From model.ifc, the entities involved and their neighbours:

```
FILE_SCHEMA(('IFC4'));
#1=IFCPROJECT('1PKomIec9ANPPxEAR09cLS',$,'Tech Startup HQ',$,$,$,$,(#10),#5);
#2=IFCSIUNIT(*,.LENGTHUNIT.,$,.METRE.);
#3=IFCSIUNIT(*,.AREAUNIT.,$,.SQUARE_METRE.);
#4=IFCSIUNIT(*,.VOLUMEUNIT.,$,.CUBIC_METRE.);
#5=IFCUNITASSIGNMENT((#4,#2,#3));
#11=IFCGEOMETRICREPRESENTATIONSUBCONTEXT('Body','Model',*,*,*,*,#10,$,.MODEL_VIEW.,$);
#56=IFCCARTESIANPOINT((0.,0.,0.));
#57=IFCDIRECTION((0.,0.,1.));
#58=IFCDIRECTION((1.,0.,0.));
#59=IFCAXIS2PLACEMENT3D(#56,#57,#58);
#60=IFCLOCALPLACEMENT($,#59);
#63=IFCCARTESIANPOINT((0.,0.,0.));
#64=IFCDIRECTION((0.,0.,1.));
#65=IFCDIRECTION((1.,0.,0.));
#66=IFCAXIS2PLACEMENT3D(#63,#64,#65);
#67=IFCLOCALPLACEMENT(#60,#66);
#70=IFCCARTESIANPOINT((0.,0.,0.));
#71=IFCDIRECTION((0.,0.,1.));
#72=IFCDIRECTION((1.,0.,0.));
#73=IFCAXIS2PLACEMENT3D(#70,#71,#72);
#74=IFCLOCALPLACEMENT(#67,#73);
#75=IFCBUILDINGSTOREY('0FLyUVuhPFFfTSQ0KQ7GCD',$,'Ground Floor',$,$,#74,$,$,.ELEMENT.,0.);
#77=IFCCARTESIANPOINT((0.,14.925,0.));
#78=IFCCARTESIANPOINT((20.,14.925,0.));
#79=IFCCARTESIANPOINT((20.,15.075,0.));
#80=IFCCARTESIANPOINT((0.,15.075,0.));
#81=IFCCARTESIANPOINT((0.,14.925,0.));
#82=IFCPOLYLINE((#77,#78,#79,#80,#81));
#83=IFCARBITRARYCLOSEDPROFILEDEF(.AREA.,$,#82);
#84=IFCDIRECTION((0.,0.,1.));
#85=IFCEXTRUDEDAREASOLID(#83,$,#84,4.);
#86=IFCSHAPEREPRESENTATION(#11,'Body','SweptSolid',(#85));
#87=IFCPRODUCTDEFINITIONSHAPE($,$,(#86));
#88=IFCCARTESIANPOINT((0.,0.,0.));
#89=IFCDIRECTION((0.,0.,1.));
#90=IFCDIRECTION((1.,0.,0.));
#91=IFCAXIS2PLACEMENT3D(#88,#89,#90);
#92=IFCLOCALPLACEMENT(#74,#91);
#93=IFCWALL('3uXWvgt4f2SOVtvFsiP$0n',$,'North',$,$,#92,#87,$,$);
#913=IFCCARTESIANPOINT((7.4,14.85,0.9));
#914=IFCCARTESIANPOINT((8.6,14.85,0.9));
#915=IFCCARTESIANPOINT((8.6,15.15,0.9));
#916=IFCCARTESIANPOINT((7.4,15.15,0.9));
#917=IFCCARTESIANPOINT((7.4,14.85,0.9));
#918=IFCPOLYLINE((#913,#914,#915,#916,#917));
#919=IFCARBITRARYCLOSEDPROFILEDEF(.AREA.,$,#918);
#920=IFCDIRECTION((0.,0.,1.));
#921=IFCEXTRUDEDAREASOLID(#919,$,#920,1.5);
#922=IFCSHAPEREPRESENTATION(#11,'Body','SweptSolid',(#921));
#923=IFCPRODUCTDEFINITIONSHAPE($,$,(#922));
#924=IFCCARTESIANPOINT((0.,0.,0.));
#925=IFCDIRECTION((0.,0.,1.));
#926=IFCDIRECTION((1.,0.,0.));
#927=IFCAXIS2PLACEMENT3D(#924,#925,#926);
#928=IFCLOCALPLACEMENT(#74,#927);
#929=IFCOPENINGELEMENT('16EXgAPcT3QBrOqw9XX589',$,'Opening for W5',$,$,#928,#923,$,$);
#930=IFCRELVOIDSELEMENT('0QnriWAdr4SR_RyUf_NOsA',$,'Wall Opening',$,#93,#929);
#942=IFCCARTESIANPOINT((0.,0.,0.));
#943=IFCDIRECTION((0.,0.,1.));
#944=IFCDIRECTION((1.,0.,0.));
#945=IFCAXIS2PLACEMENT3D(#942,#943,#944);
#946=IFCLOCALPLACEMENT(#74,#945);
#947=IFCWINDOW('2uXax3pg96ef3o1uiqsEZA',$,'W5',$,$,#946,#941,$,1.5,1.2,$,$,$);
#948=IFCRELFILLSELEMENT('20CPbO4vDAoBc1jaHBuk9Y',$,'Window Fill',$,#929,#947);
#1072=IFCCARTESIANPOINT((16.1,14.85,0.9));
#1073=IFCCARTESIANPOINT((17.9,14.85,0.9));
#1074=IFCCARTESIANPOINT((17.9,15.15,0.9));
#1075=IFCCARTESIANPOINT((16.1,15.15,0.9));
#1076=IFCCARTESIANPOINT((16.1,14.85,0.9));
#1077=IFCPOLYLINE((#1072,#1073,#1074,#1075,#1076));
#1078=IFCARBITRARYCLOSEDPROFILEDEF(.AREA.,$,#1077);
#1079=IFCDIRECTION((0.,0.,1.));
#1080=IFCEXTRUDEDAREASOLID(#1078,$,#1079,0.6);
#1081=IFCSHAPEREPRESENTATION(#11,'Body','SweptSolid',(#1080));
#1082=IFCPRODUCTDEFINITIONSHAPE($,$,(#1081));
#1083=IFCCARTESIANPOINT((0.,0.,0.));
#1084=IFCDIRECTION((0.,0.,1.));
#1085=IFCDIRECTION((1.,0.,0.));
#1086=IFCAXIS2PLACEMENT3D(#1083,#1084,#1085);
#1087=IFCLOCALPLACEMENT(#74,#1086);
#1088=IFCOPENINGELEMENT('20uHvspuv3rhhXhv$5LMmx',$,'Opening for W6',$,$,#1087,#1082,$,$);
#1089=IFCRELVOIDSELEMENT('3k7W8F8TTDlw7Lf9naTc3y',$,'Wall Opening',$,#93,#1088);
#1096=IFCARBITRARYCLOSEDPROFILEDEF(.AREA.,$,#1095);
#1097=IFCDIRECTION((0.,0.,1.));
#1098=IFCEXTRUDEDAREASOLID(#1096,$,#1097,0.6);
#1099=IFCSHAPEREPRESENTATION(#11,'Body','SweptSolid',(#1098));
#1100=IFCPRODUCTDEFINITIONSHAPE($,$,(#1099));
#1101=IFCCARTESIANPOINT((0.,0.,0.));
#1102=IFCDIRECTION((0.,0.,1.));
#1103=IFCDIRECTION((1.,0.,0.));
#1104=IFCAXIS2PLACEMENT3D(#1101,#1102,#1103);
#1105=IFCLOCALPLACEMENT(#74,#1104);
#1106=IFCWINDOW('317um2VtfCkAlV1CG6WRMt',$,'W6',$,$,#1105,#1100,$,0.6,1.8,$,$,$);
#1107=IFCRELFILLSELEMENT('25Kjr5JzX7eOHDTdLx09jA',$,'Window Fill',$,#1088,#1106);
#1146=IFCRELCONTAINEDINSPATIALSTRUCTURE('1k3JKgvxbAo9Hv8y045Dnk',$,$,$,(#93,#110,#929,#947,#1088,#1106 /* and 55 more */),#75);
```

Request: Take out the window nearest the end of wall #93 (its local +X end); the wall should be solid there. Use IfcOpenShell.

```python
import ifcopenshell
import ifcopenshell.api.feature
import ifcopenshell.api.root
import ifcopenshell.geom
import ifcopenshell.util.shape

model = ifcopenshell.open("model.ifc")
settings = ifcopenshell.geom.settings()


def volume(element):
    """Net volume in cubic metres, openings subtracted."""
    shape = ifcopenshell.geom.create_shape(settings, element)
    return ifcopenshell.util.shape.get_volume(shape.geometry)


window = model.by_guid("317um2VtfCkAlV1CG6WRMt")
opening = window.FillsVoids[0].RelatingOpeningElement
wall = opening.VoidsElements[0].RelatingBuildingElement
before = volume(wall)

ifcopenshell.api.root.remove_product(model, product=window)
ifcopenshell.api.feature.remove_feature(model, feature=opening)

after = volume(wall)

print(f"wall volume {before:.3f} -> {after:.3f} m3")

model.write("model_v2.ifc")
```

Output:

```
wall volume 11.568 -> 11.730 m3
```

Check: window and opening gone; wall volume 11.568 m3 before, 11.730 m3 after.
